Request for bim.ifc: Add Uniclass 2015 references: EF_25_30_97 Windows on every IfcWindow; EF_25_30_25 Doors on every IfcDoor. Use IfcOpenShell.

First a look at what the model holds.

```python
import ifcopenshell

model = ifcopenshell.open("bim.ifc")
print(model.schema)
print("classifications:", [c.Name for c in model.by_type("IfcClassification")])
for ifc_class in ("IfcDoor", "IfcRoof", "IfcStair", "IfcWall", "IfcWindow"):
    print(ifc_class, len(model.by_type(ifc_class)))
```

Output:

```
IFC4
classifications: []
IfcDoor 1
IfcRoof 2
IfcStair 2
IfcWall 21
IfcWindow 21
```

```python
import ifcopenshell
import ifcopenshell.api.classification

model = ifcopenshell.open("bim.ifc")

system = ifcopenshell.api.classification.add_classification(model, classification="Uniclass 2015")

codes = {
    "IfcWindow": ("EF_25_30_97", "Windows"),
    "IfcDoor": ("EF_25_30_25", "Doors"),
}
for ifc_class, (code, name) in codes.items():
    products = model.by_type(ifc_class)
    ifcopenshell.api.classification.add_reference(
        model, products=products, classification=system, identification=code, name=name
    )
    print(code, len(products))

model.write("bim_rev.ifc")
```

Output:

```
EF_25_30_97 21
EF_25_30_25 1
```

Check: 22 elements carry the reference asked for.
